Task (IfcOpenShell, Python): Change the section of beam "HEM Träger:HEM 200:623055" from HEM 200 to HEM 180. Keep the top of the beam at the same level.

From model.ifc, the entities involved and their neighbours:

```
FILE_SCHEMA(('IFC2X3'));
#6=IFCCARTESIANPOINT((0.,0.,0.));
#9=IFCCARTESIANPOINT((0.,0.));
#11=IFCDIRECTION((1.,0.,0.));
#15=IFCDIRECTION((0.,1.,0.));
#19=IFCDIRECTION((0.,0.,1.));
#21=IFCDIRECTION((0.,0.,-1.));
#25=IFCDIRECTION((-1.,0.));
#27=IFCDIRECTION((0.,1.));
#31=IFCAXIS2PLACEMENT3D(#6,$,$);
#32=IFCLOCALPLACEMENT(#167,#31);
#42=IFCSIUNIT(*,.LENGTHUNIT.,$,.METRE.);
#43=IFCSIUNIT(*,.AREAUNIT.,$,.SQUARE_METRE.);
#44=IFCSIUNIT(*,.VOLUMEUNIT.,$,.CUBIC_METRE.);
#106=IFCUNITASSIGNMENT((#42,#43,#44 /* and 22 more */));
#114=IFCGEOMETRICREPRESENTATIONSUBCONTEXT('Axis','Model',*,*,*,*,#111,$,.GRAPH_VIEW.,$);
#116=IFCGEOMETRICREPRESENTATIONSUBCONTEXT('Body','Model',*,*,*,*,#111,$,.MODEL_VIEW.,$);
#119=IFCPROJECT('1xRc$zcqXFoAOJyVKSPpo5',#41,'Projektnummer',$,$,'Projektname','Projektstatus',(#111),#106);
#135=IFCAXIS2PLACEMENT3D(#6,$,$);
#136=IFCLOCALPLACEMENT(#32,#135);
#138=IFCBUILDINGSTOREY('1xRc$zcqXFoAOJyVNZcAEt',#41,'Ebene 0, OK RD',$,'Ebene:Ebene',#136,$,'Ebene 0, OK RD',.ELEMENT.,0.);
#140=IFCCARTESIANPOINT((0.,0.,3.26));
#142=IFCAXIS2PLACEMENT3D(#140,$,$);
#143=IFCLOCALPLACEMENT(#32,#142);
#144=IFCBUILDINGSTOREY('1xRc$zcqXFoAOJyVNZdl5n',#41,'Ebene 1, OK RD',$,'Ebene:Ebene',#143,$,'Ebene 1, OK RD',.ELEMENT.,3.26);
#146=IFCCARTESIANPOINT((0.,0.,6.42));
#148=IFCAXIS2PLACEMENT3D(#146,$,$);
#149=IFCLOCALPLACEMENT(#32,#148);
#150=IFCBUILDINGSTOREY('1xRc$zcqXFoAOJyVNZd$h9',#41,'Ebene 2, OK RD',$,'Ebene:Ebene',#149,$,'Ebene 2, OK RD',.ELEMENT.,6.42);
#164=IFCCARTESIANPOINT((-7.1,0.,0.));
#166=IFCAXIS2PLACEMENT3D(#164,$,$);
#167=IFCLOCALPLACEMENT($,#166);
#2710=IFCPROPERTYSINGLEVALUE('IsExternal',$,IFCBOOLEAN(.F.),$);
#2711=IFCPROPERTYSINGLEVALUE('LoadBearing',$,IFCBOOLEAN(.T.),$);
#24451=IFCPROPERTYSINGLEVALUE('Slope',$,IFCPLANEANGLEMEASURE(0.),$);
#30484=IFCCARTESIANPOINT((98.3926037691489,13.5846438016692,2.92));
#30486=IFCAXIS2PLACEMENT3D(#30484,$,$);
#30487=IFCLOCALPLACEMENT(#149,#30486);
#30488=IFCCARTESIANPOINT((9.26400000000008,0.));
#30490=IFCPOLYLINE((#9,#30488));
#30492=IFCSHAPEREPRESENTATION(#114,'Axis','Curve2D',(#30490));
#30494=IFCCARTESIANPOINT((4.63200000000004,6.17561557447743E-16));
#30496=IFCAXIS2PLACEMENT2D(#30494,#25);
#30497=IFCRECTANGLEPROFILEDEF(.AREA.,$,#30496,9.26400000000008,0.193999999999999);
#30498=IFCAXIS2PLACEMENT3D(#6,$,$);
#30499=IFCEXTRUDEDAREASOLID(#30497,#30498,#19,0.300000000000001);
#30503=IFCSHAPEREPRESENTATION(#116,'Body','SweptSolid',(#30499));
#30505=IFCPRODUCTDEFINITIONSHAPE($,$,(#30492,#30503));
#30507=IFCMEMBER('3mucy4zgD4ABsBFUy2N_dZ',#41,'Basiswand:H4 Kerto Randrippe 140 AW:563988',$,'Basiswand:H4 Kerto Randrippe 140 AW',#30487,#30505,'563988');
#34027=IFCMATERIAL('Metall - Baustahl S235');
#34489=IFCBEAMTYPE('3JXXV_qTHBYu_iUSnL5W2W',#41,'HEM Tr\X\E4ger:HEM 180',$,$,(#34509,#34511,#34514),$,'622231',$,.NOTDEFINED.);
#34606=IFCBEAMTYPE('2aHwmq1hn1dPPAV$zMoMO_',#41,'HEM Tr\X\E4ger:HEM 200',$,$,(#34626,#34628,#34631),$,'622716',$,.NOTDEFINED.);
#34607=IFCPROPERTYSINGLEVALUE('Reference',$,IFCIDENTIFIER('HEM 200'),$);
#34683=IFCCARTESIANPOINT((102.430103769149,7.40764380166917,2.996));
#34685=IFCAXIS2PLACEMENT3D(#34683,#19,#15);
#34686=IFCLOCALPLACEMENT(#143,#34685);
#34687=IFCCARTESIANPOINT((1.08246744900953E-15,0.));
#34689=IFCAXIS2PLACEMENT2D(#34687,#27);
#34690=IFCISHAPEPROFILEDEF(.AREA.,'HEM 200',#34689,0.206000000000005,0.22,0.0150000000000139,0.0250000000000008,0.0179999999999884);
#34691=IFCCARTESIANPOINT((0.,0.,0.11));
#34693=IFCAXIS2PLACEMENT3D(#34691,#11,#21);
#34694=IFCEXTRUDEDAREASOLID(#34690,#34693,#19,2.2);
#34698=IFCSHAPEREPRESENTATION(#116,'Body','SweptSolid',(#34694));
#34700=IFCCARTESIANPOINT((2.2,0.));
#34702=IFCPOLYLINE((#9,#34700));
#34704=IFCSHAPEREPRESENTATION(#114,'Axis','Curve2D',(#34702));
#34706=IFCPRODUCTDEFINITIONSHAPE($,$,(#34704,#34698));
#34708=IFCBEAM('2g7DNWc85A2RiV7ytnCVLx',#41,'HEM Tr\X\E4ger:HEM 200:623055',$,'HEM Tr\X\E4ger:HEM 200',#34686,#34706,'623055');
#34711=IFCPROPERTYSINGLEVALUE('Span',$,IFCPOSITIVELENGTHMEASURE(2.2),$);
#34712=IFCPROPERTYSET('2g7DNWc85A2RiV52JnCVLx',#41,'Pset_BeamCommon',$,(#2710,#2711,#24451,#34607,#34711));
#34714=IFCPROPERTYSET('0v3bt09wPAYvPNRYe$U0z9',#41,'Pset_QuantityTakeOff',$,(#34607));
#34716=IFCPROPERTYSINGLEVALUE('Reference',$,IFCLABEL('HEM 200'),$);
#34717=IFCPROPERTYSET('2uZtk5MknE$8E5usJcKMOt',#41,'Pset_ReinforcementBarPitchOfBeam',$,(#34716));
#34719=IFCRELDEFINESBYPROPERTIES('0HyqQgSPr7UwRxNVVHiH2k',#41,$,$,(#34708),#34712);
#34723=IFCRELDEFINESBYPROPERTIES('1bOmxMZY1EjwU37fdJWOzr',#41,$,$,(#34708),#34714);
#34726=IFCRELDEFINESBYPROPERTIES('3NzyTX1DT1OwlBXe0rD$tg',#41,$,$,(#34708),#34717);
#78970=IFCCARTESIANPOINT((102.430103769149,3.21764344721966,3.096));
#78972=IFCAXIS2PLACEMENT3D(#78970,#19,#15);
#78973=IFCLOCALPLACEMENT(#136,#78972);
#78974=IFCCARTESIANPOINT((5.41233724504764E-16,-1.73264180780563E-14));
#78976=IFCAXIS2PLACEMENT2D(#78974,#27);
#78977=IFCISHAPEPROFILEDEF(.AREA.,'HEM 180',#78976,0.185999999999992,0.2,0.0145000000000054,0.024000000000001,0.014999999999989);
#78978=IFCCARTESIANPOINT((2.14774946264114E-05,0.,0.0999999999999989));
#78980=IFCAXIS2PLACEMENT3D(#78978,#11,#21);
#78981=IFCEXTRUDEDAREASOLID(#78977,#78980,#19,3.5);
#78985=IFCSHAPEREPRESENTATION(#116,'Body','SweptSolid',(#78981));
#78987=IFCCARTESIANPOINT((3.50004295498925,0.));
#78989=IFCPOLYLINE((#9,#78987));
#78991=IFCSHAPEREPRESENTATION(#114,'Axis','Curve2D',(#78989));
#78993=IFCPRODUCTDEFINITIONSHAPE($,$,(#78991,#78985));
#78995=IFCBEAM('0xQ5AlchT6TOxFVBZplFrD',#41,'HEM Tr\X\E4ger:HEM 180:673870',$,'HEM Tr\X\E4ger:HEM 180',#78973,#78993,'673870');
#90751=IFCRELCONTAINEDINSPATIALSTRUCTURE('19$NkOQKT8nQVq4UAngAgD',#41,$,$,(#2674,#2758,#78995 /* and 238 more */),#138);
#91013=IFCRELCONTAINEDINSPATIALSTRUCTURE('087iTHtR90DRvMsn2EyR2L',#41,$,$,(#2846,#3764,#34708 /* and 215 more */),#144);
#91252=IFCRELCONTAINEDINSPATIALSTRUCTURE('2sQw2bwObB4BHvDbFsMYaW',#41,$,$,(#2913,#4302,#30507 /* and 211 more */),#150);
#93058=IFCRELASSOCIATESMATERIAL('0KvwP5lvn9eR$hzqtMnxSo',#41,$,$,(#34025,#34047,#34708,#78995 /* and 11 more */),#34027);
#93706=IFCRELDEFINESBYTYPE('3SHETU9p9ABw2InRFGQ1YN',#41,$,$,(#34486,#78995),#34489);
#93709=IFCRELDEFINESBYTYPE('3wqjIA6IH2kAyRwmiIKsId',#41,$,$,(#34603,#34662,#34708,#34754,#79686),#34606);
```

```python
import ifcopenshell
import ifcopenshell.api.pset
import ifcopenshell.api.type
import ifcopenshell.util.element
import ifcopenshell.util.representation

model = ifcopenshell.open("model.ifc")

member = model.by_guid("2g7DNWc85A2RiV7ytnCVLx")
source = next(p for p in model.by_type("IfcIShapeProfileDef") if p.ProfileName == "HEM 180")

body = ifcopenshell.util.representation.get_representation(member, "Model", "Body")
solid = body.Items[0]
old_profile = solid.SweptArea

# Copy the section's sizes but keep this member's own profile position.
profile = ifcopenshell.util.element.copy(model, source)
# Profiles are centred, so shift by half the change in depth to hold the top.
shift = (old_profile.OverallDepth - profile.OverallDepth) / 2
x, y = old_profile.Position.Location.Coordinates
up = (-1.0, 0.0)  # upwards, in the solid's own plane
location = model.createIfcCartesianPoint((x + up[0] * shift, y + up[1] * shift))
profile.Position = model.createIfcAxis2Placement2D(location, old_profile.Position.RefDirection)
solid.SweptArea = profile
if not model.get_total_inverses(old_profile):
    ifcopenshell.util.element.remove_deep2(model, old_profile)

new_type = model.by_guid("3JXXV_qTHBYu_iUSnL5W2W")
ifcopenshell.api.type.assign_type(
    model, related_objects=[member], relating_type=new_type, should_map_representations=False
)
member.Name = member.Name.replace("HEM 200", "HEM 180")
member.ObjectType = "HEM Träger:HEM 180"
pset = model.by_id(ifcopenshell.util.element.get_pset(member, "Pset_BeamCommon", should_inherit=False)["id"])
ifcopenshell.api.pset.edit_pset(model, pset=pset, properties={"Reference": "HEM 180"})
pset = model.by_id(ifcopenshell.util.element.get_pset(member, "Pset_QuantityTakeOff", should_inherit=False)["id"])
ifcopenshell.api.pset.edit_pset(model, pset=pset, properties={"Reference": "HEM 180"})
pset = model.by_id(ifcopenshell.util.element.get_pset(member, "Pset_ReinforcementBarPitchOfBeam", should_inherit=False)["id"])
ifcopenshell.api.pset.edit_pset(model, pset=pset, properties={"Reference": "HEM 180"})

print(solid.SweptArea)

model.write("model_updated.ifc")
```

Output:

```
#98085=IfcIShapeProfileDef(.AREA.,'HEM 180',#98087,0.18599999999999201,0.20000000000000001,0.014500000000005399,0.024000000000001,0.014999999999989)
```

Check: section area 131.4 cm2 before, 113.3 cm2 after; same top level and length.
